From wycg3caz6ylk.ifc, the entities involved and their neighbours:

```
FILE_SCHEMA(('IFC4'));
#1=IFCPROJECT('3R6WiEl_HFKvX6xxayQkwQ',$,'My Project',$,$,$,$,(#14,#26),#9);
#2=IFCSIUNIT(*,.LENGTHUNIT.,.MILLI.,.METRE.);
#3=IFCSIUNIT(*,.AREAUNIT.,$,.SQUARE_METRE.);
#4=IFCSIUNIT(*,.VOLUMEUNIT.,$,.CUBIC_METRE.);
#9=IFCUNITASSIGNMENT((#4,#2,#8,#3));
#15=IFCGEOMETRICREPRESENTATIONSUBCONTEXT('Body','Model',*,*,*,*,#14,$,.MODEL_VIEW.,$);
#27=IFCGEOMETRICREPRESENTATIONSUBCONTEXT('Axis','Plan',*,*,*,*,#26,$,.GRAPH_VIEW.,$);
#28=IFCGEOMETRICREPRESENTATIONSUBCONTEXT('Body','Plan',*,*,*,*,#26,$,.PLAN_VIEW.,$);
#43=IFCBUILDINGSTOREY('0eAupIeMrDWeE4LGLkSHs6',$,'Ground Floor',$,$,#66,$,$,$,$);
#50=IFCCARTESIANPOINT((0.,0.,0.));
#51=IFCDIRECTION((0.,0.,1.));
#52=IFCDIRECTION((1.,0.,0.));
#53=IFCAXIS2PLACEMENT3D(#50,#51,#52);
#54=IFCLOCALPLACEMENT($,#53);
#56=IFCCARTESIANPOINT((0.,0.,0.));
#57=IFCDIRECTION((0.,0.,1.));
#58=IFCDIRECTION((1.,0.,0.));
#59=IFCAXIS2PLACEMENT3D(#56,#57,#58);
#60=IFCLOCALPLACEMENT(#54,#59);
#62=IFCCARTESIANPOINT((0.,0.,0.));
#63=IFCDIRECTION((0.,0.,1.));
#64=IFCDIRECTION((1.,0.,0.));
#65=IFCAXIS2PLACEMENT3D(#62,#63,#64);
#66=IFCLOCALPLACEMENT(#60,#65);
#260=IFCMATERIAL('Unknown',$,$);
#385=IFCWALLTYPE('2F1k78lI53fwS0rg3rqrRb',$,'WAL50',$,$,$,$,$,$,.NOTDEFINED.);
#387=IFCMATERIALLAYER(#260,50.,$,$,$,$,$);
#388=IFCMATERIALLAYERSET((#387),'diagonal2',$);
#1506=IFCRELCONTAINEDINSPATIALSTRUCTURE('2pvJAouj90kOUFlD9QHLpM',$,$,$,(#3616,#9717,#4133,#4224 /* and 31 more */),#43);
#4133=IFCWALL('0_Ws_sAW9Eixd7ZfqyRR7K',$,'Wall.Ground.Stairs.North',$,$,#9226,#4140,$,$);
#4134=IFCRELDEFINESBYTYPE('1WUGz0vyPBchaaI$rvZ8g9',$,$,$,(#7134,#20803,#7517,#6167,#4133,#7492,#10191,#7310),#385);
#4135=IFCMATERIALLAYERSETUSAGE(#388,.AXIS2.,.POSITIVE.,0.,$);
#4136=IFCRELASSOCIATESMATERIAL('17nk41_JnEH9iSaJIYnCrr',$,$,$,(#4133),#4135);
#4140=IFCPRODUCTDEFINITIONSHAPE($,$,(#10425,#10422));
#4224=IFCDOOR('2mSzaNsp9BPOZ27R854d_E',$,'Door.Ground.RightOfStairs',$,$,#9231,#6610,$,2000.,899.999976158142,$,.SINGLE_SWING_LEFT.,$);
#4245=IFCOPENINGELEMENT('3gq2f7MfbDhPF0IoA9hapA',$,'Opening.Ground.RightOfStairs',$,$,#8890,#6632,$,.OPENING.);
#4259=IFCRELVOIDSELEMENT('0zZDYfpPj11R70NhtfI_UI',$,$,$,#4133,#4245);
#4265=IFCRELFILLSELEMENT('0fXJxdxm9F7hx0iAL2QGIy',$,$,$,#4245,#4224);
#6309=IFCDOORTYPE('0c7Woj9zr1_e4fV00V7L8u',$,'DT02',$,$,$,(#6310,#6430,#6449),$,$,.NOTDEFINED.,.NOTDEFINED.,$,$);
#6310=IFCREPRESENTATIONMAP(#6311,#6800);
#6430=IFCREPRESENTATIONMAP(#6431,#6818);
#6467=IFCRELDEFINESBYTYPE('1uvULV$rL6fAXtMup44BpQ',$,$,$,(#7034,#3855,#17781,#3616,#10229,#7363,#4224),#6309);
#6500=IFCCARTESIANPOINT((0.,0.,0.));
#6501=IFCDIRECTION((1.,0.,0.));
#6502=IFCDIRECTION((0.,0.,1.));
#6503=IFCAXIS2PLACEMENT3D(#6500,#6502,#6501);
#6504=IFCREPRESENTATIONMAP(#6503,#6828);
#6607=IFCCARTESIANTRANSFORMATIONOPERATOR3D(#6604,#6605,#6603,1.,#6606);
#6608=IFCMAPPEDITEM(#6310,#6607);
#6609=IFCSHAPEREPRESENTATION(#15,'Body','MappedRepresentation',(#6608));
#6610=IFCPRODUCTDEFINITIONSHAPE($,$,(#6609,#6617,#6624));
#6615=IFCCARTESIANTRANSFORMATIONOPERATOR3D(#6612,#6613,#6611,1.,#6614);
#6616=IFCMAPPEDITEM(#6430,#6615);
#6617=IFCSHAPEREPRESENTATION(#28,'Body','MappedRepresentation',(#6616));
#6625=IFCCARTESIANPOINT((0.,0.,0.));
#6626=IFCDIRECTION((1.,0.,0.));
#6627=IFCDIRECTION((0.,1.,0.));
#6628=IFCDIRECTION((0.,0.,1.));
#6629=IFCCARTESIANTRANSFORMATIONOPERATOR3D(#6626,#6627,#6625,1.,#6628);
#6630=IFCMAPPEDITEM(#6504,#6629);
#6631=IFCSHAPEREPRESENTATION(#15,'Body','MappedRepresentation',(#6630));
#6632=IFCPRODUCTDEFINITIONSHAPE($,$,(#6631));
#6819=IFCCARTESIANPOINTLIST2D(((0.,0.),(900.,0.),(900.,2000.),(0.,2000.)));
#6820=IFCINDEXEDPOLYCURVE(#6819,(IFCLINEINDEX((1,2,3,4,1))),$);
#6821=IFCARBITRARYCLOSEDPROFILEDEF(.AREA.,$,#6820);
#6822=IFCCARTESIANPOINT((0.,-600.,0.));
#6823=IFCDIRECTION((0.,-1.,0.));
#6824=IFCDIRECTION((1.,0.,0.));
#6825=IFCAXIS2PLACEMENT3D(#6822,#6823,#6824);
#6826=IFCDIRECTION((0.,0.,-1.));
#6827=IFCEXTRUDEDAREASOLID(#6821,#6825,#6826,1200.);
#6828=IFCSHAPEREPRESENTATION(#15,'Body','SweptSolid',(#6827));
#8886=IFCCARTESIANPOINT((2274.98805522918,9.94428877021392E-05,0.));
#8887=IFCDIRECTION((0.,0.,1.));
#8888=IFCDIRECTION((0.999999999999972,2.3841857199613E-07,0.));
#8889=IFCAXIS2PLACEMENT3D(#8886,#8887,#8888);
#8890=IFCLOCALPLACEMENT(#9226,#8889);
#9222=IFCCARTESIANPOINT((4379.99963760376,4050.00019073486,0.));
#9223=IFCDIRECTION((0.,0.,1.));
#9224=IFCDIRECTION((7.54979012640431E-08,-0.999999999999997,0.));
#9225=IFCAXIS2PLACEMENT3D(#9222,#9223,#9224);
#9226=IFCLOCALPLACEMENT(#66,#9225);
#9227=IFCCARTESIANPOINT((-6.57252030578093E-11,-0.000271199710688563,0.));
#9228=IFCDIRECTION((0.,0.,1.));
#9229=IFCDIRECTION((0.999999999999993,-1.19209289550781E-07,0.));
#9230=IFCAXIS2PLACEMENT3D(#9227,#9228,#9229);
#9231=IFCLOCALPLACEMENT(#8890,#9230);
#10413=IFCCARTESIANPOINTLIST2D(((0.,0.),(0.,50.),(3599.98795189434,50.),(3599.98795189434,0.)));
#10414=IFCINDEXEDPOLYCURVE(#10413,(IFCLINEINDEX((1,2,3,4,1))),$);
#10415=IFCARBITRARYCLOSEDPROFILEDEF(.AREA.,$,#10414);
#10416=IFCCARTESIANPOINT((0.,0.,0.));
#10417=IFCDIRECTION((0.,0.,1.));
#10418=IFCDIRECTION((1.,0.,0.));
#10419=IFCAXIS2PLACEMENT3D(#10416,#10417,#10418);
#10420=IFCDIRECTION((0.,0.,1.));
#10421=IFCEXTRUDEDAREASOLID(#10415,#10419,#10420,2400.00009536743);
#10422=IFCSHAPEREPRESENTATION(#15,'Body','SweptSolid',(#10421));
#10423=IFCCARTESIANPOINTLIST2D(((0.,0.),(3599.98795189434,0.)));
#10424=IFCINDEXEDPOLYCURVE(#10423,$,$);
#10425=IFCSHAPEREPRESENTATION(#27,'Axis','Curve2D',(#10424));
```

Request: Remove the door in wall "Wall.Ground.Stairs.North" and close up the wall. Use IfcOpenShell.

```python
import ifcopenshell
import ifcopenshell.api.feature
import ifcopenshell.api.root
import ifcopenshell.geom
import ifcopenshell.util.shape

model = ifcopenshell.open("wycg3caz6ylk.ifc")
settings = ifcopenshell.geom.settings()


def volume(element):
    """Net volume in cubic metres, openings subtracted."""
    shape = ifcopenshell.geom.create_shape(settings, element)
    return ifcopenshell.util.shape.get_volume(shape.geometry)


door = model.by_id(4224)
opening = door.FillsVoids[0].RelatingOpeningElement
wall = opening.VoidsElements[0].RelatingBuildingElement
before = volume(wall)

ifcopenshell.api.root.remove_product(model, product=door)
ifcopenshell.api.feature.remove_feature(model, feature=opening)

after = volume(wall)

print(f"wall volume {before:.3f} -> {after:.3f} m3")

model.write("wycg3caz6ylk_rev.ifc")
```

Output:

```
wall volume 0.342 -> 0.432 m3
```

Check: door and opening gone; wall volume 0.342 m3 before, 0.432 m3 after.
